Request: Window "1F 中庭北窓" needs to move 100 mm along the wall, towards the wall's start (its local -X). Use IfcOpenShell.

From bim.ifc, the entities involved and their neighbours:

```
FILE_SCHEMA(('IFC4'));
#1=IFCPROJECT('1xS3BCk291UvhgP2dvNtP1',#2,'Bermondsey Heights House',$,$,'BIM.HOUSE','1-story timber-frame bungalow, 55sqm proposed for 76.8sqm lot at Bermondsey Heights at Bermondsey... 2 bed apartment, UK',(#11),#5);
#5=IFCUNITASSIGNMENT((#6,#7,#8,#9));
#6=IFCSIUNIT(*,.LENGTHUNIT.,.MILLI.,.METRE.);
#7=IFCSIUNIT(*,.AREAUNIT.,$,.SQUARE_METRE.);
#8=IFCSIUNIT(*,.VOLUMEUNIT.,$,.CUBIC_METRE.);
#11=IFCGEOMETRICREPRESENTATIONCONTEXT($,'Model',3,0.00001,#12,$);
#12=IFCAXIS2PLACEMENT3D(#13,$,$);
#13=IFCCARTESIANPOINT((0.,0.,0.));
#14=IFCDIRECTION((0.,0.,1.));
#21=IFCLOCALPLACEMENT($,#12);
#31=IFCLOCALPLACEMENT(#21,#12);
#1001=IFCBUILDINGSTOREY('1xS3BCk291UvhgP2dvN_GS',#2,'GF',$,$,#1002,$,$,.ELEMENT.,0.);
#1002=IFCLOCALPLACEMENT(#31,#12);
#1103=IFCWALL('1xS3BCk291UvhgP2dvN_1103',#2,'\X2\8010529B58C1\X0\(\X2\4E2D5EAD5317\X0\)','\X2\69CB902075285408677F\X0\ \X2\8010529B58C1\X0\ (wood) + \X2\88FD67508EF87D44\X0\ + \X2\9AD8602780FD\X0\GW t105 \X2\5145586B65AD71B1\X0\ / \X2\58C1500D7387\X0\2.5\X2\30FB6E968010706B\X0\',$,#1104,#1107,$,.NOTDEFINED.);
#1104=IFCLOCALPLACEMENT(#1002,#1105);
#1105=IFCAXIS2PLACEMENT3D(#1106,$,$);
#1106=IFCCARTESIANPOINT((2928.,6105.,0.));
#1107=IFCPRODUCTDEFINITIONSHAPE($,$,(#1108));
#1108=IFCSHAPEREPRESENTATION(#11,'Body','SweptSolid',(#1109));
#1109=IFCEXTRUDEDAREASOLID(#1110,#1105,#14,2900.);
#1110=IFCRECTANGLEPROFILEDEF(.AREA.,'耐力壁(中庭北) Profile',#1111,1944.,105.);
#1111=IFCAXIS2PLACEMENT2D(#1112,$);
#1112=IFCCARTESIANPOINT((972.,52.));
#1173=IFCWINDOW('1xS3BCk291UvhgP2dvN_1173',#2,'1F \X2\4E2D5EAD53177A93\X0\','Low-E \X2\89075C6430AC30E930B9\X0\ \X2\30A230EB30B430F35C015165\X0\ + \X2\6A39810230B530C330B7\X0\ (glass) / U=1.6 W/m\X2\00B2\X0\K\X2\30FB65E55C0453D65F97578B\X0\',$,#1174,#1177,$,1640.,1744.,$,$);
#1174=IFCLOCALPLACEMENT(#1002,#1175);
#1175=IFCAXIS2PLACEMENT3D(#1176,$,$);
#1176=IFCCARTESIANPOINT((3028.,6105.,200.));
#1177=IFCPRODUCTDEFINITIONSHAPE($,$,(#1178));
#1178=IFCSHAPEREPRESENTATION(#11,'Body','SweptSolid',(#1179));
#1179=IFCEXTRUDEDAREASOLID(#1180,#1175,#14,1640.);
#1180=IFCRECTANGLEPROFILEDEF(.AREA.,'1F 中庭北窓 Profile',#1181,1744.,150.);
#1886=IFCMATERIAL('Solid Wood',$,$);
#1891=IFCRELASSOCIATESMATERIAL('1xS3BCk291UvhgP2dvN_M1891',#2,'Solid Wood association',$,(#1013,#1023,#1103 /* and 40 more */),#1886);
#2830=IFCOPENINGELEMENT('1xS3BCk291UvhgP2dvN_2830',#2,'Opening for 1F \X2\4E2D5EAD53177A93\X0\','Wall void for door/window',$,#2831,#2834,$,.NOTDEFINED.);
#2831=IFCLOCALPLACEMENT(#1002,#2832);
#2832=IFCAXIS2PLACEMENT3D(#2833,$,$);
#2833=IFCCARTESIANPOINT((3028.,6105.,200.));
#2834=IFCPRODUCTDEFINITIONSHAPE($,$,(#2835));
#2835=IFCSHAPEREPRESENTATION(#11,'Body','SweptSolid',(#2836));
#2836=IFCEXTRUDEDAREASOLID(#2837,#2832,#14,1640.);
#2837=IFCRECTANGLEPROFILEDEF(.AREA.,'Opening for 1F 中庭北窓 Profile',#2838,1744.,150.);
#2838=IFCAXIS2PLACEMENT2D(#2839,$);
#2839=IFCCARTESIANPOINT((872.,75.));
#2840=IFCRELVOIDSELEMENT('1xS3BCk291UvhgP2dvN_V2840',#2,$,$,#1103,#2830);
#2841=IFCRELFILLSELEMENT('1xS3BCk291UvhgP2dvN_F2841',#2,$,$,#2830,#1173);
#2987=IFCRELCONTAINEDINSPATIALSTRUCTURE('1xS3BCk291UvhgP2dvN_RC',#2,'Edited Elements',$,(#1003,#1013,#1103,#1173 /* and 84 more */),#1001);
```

```python
import ifcopenshell
import ifcopenshell.api.geometry
import ifcopenshell.util.placement
import ifcopenshell.util.unit

model = ifcopenshell.open("bim.ifc")
unit_scale = ifcopenshell.util.unit.calculate_unit_scale(model)

window = model.by_id(1173)
opening = window.FillsVoids[0].RelatingOpeningElement
wall = opening.VoidsElements[0].RelatingBuildingElement

wall_matrix = ifcopenshell.util.placement.get_local_placement(wall.ObjectPlacement)
shift = wall_matrix[:3, 0] * -0.1 / unit_scale
before = ifcopenshell.util.placement.get_local_placement(window.ObjectPlacement)[:3, 3].copy()

# The window is not placed relative to its opening, so move both.
for product in (opening, window):
    matrix = ifcopenshell.util.placement.get_local_placement(product.ObjectPlacement)
    matrix[:3, 3] += shift
    ifcopenshell.api.geometry.edit_object_placement(model, product=product, matrix=matrix, is_si=False)

after = ifcopenshell.util.placement.get_local_placement(window.ObjectPlacement)[:3, 3]
print("window moved by", (after - before).round(3) + 0.0)

model.write("bim_rev.ifc")
```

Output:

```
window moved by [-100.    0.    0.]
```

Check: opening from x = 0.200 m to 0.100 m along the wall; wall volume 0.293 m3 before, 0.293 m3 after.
